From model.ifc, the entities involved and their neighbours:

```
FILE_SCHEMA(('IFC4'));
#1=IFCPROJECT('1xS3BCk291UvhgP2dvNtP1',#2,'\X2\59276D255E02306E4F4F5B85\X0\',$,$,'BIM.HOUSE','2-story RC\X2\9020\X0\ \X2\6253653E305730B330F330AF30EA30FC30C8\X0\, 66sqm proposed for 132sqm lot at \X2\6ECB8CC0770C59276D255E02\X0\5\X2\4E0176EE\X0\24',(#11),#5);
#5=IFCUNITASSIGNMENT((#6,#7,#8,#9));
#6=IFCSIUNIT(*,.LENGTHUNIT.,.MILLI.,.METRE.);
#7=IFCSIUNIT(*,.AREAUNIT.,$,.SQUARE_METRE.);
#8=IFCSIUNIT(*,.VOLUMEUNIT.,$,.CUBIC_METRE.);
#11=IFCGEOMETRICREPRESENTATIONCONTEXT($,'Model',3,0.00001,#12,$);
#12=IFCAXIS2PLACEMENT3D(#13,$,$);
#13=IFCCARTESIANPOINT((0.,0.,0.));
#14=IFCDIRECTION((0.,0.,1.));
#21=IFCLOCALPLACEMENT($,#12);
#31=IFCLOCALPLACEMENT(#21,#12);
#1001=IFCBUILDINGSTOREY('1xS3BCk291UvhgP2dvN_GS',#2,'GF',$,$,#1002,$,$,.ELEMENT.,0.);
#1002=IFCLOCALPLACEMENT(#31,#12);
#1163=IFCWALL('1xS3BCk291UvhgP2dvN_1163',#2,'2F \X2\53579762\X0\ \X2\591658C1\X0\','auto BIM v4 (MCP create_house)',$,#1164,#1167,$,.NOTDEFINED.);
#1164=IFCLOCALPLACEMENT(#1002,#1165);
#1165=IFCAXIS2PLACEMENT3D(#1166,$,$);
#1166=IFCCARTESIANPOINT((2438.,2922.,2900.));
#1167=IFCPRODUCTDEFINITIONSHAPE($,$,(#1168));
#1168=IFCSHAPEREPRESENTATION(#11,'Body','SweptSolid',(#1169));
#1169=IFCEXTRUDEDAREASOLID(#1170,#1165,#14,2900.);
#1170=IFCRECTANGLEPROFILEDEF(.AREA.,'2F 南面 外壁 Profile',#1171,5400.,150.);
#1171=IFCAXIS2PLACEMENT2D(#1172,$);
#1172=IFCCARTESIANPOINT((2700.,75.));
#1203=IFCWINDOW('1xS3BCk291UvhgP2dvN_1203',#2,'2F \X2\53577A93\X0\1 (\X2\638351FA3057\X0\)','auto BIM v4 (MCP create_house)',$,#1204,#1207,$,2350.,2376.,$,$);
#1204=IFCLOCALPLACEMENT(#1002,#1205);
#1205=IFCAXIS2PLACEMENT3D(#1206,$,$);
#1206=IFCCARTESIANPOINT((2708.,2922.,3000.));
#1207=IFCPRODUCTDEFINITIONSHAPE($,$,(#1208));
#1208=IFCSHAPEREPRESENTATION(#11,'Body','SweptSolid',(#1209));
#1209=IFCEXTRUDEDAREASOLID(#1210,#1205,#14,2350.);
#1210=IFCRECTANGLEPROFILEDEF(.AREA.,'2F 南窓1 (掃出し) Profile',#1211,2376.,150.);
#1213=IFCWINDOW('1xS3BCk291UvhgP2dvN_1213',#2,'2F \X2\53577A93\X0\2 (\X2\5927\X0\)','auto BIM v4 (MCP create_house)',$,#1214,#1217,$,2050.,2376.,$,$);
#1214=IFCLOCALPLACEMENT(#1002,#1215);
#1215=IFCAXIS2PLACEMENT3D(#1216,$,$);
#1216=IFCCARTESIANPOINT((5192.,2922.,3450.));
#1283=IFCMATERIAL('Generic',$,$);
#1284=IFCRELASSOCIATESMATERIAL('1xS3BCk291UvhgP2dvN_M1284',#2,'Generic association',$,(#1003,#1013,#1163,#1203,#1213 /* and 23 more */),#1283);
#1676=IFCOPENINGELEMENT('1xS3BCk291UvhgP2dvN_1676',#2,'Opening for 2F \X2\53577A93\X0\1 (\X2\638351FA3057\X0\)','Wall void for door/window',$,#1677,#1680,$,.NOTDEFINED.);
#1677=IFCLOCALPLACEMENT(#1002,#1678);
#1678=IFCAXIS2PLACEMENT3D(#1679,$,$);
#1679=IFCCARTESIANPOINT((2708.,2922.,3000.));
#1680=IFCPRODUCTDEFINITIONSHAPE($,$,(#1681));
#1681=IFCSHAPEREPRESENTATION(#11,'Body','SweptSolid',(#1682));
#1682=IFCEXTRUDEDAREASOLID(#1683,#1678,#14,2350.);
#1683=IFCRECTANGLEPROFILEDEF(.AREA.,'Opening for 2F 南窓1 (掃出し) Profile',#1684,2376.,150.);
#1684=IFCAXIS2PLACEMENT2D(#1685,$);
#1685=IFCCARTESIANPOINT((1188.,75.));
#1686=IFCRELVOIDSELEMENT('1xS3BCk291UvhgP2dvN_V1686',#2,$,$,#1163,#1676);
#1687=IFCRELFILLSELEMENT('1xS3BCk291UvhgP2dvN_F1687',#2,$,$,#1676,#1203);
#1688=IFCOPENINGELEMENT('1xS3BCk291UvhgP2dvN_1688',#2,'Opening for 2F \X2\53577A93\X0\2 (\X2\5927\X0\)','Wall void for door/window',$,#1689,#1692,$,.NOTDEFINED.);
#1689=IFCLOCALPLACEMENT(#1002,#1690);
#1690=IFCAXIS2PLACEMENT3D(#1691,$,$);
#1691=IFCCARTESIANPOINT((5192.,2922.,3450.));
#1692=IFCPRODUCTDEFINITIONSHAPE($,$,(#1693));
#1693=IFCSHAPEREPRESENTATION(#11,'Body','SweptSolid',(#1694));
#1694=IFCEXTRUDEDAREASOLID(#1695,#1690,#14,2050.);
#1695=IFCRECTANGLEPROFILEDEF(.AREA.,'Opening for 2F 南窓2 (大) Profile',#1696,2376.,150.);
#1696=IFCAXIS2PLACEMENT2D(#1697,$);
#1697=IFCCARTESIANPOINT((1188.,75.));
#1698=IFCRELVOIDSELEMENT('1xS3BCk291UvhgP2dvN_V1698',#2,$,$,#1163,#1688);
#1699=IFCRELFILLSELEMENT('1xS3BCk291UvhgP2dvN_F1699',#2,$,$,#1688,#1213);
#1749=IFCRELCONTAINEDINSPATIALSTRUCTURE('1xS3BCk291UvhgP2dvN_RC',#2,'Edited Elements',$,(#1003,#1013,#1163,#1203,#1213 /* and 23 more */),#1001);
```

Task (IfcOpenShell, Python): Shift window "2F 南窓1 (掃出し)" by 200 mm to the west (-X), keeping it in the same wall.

```python
import ifcopenshell
import ifcopenshell.api.geometry
import ifcopenshell.util.placement

model = ifcopenshell.open("model.ifc")

window = model.by_guid("1xS3BCk291UvhgP2dvN_1203")
opening = window.FillsVoids[0].RelatingOpeningElement
wall = opening.VoidsElements[0].RelatingBuildingElement

wall_matrix = ifcopenshell.util.placement.get_local_placement(wall.ObjectPlacement)
shift = wall_matrix[:3, 0] * -200.0
before = ifcopenshell.util.placement.get_local_placement(window.ObjectPlacement)[:3, 3].copy()

# The window is not placed relative to its opening, so move both.
for product in (opening, window):
    matrix = ifcopenshell.util.placement.get_local_placement(product.ObjectPlacement)
    matrix[:3, 3] += shift
    ifcopenshell.api.geometry.edit_object_placement(model, product=product, matrix=matrix, is_si=False)

after = ifcopenshell.util.placement.get_local_placement(window.ObjectPlacement)[:3, 3]
print("window moved by", (after - before).round(3) + 0.0)

model.write("model_edited.ifc")
```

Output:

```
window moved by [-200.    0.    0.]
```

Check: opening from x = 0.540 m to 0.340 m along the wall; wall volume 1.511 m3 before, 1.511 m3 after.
